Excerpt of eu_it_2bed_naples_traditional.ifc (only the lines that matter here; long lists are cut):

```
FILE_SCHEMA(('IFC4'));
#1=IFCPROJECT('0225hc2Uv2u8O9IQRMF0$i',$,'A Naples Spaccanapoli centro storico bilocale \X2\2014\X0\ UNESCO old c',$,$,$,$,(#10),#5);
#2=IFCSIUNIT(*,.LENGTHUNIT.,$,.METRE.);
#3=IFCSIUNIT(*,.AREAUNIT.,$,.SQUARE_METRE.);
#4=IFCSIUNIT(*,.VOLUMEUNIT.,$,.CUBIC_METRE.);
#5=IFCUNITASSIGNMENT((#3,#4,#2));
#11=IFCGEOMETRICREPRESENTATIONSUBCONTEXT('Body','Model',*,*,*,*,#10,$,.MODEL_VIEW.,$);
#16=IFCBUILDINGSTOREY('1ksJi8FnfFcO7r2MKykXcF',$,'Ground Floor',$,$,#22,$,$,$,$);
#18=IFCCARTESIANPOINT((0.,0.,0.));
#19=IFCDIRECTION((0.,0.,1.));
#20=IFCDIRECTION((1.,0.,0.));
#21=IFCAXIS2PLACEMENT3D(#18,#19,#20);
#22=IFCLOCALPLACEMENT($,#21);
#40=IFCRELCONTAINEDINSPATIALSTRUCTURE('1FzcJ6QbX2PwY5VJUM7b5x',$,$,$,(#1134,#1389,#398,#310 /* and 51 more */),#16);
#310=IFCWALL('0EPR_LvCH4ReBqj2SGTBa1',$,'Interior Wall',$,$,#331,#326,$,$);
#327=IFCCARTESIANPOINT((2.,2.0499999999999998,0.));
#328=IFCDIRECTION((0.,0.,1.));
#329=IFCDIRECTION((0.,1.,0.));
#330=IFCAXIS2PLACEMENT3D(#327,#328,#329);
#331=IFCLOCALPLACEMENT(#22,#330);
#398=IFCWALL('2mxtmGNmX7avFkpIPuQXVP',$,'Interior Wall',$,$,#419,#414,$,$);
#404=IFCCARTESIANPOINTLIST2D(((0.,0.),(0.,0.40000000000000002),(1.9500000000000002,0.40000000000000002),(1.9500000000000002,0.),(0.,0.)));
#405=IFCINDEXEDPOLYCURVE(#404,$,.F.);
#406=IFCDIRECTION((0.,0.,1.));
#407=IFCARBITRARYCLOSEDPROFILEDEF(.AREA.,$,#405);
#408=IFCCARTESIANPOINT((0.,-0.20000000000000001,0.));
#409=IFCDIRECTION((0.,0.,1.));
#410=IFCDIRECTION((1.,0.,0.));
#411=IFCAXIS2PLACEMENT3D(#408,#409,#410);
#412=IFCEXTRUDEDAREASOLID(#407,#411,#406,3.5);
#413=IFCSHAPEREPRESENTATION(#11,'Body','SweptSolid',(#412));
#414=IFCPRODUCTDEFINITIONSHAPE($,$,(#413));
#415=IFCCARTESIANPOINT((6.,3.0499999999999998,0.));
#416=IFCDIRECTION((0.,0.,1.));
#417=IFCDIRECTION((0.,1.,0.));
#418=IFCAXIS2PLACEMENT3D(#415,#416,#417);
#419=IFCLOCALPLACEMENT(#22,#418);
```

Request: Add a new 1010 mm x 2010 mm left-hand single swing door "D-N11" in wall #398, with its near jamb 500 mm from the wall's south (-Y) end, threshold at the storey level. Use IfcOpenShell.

```python
import numpy as np
import ifcopenshell
import ifcopenshell.api.feature
import ifcopenshell.api.geometry
import ifcopenshell.api.root
import ifcopenshell.api.spatial
import ifcopenshell.geom
import ifcopenshell.util.element
import ifcopenshell.util.placement
import ifcopenshell.util.representation
import ifcopenshell.util.shape
import ifcopenshell.util.unit

model = ifcopenshell.open("eu_it_2bed_naples_traditional.ifc")
unit_scale = ifcopenshell.util.unit.calculate_unit_scale(model)
settings = ifcopenshell.geom.settings()


def volume(element):
    """Net volume in cubic metres, openings subtracted."""
    shape = ifcopenshell.geom.create_shape(settings, element)
    return ifcopenshell.util.shape.get_volume(shape.geometry)


wall = model.by_id(398)
storey = ifcopenshell.util.element.get_container(wall, ifc_class="IfcBuildingStorey")
context = ifcopenshell.util.representation.get_context(model, "Model", "Body", "MODEL_VIEW")
before = volume(wall)

width, height, from_end, sill = 1.01, 2.01, 0.5, 0.0  # metres

# The wall runs along its own X axis, and the end named is its -X end.
wall_shape = ifcopenshell.geom.create_shape(settings, wall)
x, y, z = ifcopenshell.util.shape.get_vertices(wall_shape.geometry).T
start = x.min() + from_end
face, thickness = float(y.min()), float(y.max() - y.min())
wall_matrix = ifcopenshell.util.placement.get_local_placement(wall.ObjectPlacement)
level = ifcopenshell.util.placement.get_local_placement(storey.ObjectPlacement)[2, 3]


def in_wall(x, y):
    """Placement at x, y metres in the wall's axes, at sill height."""
    matrix = wall_matrix.copy()
    matrix[:, 3] = wall_matrix @ np.array([x / unit_scale, y / unit_scale, 0.0, 1.0])
    matrix[2, 3] = level + sill / unit_scale
    return matrix


# Opening: a box that overshoots both wall faces by 50 mm.
opening = ifcopenshell.api.root.create_entity(model, ifc_class="IfcOpeningElement", predefined_type="OPENING")
box = ifcopenshell.api.geometry.add_wall_representation(
    model, context=context, length=width, height=height, thickness=thickness + 0.1
)
ifcopenshell.api.geometry.assign_representation(model, product=opening, representation=box)
ifcopenshell.api.geometry.edit_object_placement(model, product=opening, matrix=in_wall(start, face - 0.05), is_si=False)
ifcopenshell.api.feature.add_feature(model, feature=opening, element=wall)

door = ifcopenshell.api.root.create_entity(model, ifc_class="IfcDoor", name="D-N11", predefined_type="DOOR")
door.OverallWidth, door.OverallHeight = width / unit_scale, height / unit_scale
door.OperationType = "SINGLE_SWING_LEFT"
body = ifcopenshell.api.geometry.add_door_representation(
    model,
    context=context,
    overall_width=door.OverallWidth,
    overall_height=door.OverallHeight,
    operation_type="SINGLE_SWING_LEFT",
    lining_properties={"LiningDepth": thickness / unit_scale, "ThresholdDepth": thickness / unit_scale},
)
ifcopenshell.api.geometry.assign_representation(model, product=door, representation=body)
ifcopenshell.api.spatial.assign_container(model, products=[door], relating_structure=storey)
ifcopenshell.api.feature.add_filling(model, opening=opening, element=door)

# The lining spans the wall, so the door starts at the wall face.
ifcopenshell.api.geometry.edit_object_placement(model, product=door, matrix=in_wall(start, face), is_si=False)

after = volume(wall)

print(f"wall volume {before:.3f} -> {after:.3f} m3")

model.write("eu_it_2bed_naples_traditional_rev.ifc")
```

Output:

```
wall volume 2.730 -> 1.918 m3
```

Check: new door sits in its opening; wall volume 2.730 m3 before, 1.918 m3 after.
